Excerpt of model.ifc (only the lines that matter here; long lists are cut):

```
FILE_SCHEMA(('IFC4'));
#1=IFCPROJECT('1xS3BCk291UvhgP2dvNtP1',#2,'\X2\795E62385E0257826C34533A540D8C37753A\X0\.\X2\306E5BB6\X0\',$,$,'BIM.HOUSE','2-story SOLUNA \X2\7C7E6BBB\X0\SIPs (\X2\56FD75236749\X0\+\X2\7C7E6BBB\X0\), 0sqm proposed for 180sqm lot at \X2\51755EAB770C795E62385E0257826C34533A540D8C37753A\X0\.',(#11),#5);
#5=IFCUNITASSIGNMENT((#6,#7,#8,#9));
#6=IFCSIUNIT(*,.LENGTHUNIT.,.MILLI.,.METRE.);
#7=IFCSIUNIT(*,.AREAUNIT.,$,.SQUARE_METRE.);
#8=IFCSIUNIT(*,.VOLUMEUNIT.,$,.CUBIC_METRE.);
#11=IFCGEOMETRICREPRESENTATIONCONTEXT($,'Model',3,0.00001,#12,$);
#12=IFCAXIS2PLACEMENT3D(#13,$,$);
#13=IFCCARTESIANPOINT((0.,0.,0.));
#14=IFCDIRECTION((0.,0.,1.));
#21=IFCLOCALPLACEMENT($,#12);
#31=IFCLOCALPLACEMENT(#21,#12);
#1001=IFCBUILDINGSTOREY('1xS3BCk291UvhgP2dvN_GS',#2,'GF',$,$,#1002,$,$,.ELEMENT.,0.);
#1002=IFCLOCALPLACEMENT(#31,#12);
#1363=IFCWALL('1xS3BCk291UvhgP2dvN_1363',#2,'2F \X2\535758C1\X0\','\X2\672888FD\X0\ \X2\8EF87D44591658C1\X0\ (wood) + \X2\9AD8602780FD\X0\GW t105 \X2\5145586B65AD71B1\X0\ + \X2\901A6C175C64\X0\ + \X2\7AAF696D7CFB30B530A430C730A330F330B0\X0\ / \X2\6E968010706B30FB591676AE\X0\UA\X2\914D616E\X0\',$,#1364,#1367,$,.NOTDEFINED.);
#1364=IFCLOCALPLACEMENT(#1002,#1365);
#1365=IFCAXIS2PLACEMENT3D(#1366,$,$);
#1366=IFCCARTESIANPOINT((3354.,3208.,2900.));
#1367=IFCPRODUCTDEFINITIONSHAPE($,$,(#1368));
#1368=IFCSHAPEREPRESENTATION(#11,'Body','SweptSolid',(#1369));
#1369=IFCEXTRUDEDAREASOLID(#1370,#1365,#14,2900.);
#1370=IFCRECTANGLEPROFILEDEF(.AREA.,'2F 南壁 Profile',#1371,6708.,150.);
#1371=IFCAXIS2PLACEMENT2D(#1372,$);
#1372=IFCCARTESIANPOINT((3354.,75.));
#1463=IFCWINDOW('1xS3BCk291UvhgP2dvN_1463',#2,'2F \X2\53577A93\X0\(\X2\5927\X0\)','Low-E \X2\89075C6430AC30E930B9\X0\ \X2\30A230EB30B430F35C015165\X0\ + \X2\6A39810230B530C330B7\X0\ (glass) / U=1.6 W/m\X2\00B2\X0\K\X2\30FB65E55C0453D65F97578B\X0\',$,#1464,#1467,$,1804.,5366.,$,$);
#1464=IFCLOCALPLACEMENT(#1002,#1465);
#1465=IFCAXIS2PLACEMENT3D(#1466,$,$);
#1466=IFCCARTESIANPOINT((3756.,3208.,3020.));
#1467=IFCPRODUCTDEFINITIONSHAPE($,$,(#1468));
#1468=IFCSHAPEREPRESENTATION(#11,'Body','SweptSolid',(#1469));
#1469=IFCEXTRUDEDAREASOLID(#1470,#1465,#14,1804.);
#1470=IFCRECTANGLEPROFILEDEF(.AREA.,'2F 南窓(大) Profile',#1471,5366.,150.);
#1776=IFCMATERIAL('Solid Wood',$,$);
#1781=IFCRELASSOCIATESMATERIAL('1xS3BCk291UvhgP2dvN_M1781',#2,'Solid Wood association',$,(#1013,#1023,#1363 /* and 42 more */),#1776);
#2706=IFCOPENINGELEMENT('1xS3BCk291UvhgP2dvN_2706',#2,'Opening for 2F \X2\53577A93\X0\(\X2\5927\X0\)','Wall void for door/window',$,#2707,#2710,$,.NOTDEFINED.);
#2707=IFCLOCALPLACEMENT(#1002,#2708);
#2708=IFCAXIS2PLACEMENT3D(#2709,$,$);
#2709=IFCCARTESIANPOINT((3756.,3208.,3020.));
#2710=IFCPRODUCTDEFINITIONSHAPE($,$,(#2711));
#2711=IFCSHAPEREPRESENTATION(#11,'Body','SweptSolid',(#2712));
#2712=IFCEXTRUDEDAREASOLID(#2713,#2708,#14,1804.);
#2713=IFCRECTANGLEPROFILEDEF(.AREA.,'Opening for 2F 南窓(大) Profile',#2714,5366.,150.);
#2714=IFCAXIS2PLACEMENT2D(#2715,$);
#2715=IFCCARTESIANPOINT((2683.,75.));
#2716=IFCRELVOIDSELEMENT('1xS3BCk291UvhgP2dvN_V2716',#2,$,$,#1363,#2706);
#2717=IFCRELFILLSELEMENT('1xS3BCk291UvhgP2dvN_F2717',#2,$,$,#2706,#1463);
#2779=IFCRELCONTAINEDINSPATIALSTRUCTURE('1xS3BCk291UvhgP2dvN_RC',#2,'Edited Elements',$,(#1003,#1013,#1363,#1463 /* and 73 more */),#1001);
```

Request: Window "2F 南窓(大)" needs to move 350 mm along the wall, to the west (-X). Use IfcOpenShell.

```python
import ifcopenshell
import ifcopenshell.api.geometry
import ifcopenshell.util.placement

model = ifcopenshell.open("model.ifc")

window = model.by_guid("1xS3BCk291UvhgP2dvN_1463")
opening = window.FillsVoids[0].RelatingOpeningElement
wall = opening.VoidsElements[0].RelatingBuildingElement

wall_matrix = ifcopenshell.util.placement.get_local_placement(wall.ObjectPlacement)
shift = wall_matrix[:3, 0] * -350.0
before = ifcopenshell.util.placement.get_local_placement(window.ObjectPlacement)[:3, 3].copy()

# The window is not placed relative to its opening, so move both.
for product in (opening, window):
    matrix = ifcopenshell.util.placement.get_local_placement(product.ObjectPlacement)
    matrix[:3, 3] += shift
    ifcopenshell.api.geometry.edit_object_placement(model, product=product, matrix=matrix, is_si=False)

after = ifcopenshell.util.placement.get_local_placement(window.ObjectPlacement)[:3, 3]
print("window moved by", (after - before).round(3) + 0.0)

model.write("model_v2.ifc")
```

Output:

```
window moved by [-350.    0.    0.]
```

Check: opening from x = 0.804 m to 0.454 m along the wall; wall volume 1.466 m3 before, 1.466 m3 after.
